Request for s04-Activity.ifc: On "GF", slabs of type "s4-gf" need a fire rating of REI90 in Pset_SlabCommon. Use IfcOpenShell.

First a look at what the model holds.

```python
import ifcopenshell
import ifcopenshell.util.element

model = ifcopenshell.open("s04-Activity.ifc")
print(model.schema)
storey = next(s for s in model.by_type("IfcBuildingStorey") if s.Name == "GF")
slabs = [e for e in ifcopenshell.util.element.get_decomposition(storey) if e.is_a("IfcSlab")]
seen = {}
for e in slabs:
    element_type = ifcopenshell.util.element.get_type(e)
    key = (element_type.Name if element_type != e and element_type else None, ifcopenshell.util.element.get_pset(e, "Pset_SlabCommon", "FireRating"))
    seen[key] = seen.get(key, 0) + 1
for (name, value), count in sorted(seen.items(), key=str):
    print(count, "x", name, "|", value)
```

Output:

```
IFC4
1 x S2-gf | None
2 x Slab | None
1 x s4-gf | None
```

```python
import ifcopenshell
import ifcopenshell.api.pset
import ifcopenshell.util.element

model = ifcopenshell.open("s04-Activity.ifc")

storey = next(s for s in model.by_type("IfcBuildingStorey") if s.Name == "GF")
slabs = [e for e in ifcopenshell.util.element.get_decomposition(storey) if e.is_a("IfcSlab")]

count = 0
for e in slabs:
    element_type = ifcopenshell.util.element.get_type(e)
    if element_type in (None, e) or element_type.Name != "s4-gf":
        continue
    # add_pset returns the element's existing set when there is one.
    pset = ifcopenshell.api.pset.add_pset(model, product=e, name="Pset_SlabCommon")
    ifcopenshell.api.pset.edit_pset(model, pset=pset, properties={"FireRating": "REI90"})
    count += 1

print(count, "slabs updated")

model.write("s04-Activity_updated.ifc")
```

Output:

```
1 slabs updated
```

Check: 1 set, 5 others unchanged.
